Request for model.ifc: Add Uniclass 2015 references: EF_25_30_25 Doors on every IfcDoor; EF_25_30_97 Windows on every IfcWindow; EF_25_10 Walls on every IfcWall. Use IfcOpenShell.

First a look at what the model holds.

```python
import ifcopenshell

model = ifcopenshell.open("model.ifc")
print(model.schema)
print("classifications:", [c.Name for c in model.by_type("IfcClassification")])
for ifc_class in ("IfcDoor", "IfcRoof", "IfcStair", "IfcWall", "IfcWindow"):
    print(ifc_class, len(model.by_type(ifc_class)))
```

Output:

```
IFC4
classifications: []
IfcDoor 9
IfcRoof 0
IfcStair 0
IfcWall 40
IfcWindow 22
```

```python
import ifcopenshell
import ifcopenshell.api.classification

model = ifcopenshell.open("model.ifc")

system = ifcopenshell.api.classification.add_classification(model, classification="Uniclass 2015")

codes = {
    "IfcDoor": ("EF_25_30_25", "Doors"),
    "IfcWindow": ("EF_25_30_97", "Windows"),
    "IfcWall": ("EF_25_10", "Walls"),
}
for ifc_class, (code, name) in codes.items():
    products = model.by_type(ifc_class)
    ifcopenshell.api.classification.add_reference(
        model, products=products, classification=system, identification=code, name=name
    )
    print(code, len(products))

model.write("model_v2.ifc")
```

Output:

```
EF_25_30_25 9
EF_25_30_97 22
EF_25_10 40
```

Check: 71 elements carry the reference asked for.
